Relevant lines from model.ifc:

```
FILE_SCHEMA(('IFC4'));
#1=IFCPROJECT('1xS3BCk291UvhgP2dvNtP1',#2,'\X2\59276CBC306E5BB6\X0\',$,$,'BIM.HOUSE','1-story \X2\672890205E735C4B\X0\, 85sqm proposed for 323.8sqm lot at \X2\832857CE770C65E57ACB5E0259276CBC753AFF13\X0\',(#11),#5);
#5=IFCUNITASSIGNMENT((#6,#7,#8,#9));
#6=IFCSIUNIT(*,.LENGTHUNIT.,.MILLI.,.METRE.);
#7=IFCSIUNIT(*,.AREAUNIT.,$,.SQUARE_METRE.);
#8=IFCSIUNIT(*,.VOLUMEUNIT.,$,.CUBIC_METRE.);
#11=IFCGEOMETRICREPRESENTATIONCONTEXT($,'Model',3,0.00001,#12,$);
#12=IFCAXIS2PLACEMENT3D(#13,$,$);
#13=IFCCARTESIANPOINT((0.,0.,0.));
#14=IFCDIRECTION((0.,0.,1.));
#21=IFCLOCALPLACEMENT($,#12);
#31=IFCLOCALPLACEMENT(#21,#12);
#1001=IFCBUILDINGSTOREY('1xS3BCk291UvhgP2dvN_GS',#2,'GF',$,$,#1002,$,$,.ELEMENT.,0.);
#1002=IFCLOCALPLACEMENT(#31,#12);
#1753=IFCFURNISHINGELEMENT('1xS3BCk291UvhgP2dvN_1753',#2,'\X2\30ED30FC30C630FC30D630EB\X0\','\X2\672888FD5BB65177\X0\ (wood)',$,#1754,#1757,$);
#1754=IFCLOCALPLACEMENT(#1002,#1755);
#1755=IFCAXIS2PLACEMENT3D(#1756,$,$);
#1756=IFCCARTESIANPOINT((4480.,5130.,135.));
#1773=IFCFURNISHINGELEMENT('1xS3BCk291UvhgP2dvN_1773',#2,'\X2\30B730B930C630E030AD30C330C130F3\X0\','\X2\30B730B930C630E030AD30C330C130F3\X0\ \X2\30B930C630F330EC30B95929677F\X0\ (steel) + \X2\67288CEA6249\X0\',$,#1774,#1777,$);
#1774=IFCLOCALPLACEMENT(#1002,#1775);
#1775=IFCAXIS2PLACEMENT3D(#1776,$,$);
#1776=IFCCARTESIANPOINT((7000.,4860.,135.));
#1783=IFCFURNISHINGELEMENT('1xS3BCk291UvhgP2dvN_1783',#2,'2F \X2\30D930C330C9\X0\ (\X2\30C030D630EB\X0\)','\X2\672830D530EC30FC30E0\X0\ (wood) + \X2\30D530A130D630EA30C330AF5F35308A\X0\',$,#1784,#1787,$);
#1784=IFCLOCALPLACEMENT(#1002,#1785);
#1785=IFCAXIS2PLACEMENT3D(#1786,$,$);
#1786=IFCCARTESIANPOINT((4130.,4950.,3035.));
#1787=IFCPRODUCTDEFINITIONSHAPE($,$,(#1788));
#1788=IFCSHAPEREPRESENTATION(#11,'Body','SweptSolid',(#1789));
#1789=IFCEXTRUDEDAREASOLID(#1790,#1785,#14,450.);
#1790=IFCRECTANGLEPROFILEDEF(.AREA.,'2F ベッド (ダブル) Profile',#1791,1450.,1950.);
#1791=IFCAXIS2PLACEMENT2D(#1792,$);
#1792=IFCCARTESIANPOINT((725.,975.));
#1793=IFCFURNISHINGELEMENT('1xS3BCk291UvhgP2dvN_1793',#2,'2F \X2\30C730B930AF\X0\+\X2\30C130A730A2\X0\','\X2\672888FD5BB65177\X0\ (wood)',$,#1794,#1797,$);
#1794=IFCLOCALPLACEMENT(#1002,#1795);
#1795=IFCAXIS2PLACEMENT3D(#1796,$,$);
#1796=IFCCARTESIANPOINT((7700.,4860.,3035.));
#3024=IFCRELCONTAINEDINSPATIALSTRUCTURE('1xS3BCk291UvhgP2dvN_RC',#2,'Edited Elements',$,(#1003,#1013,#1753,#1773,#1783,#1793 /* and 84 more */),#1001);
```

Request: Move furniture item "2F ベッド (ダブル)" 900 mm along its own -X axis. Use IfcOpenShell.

```python
import ifcopenshell
import ifcopenshell.api.geometry
import ifcopenshell.util.placement

model = ifcopenshell.open("model.ifc")

item = model.by_id(1783)
matrix = ifcopenshell.util.placement.get_local_placement(item.ObjectPlacement)
matrix[:3, 3] -= matrix[:3, 0] * 900.0
ifcopenshell.api.geometry.edit_object_placement(model, product=item, matrix=matrix, is_si=False)

print(ifcopenshell.util.placement.get_local_placement(item.ObjectPlacement).round(3) + 0.0)

model.write("model-out.ifc")
```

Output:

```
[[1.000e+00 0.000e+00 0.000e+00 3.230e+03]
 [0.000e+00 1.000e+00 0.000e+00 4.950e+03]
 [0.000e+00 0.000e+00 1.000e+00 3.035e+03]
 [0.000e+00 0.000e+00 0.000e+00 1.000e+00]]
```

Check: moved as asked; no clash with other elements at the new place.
